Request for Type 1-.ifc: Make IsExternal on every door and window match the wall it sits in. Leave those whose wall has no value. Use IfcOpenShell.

First a look at what the model holds.

```python
import ifcopenshell
import ifcopenshell.util.element

model = ifcopenshell.open("Type 1-.ifc")
print(model.schema)
seen = {}
for e in model.by_type("IfcDoor") + model.by_type("IfcWindow"):
    if not e.FillsVoids:
        continue
    host = e.FillsVoids[0].RelatingOpeningElement.VoidsElements[0].RelatingBuildingElement
    own = ifcopenshell.util.element.get_pset(e, f"Pset_{e.is_a()[3:].removesuffix('StandardCase')}Common", "IsExternal")
    wall = ifcopenshell.util.element.get_pset(host, "Pset_WallCommon", "IsExternal")
    seen[e.is_a(), own, wall] = seen.get((e.is_a(), own, wall), 0) + 1
for (cls, own, wall), count in sorted(seen.items(), key=str):
    print(count, cls, "IsExternal:", own, "| host wall:", wall)
```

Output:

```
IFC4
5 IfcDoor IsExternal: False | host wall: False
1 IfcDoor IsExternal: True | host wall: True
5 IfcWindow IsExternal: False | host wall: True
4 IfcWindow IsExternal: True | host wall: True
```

```python
import ifcopenshell
import ifcopenshell.api.pset
import ifcopenshell.util.element

model = ifcopenshell.open("Type 1-.ifc")

count = 0
for ifc_class, pset_name in (("IfcDoor", "Pset_DoorCommon"), ("IfcWindow", "Pset_WindowCommon")):
    for e in model.by_type(ifc_class):
        if not e.FillsVoids:
            continue
        host = e.FillsVoids[0].RelatingOpeningElement.VoidsElements[0].RelatingBuildingElement
        external = ifcopenshell.util.element.get_pset(host, "Pset_WallCommon", "IsExternal")
        if external is None or ifcopenshell.util.element.get_pset(e, pset_name, "IsExternal") == external:
            continue
        pset = ifcopenshell.api.pset.add_pset(model, product=e, name=pset_name)
        ifcopenshell.api.pset.edit_pset(model, pset=pset, properties={"IsExternal": external})
        count += 1

print(count, "updated")

model.write("Type 1-_rev.ifc")
```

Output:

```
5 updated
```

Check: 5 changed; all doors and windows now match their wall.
